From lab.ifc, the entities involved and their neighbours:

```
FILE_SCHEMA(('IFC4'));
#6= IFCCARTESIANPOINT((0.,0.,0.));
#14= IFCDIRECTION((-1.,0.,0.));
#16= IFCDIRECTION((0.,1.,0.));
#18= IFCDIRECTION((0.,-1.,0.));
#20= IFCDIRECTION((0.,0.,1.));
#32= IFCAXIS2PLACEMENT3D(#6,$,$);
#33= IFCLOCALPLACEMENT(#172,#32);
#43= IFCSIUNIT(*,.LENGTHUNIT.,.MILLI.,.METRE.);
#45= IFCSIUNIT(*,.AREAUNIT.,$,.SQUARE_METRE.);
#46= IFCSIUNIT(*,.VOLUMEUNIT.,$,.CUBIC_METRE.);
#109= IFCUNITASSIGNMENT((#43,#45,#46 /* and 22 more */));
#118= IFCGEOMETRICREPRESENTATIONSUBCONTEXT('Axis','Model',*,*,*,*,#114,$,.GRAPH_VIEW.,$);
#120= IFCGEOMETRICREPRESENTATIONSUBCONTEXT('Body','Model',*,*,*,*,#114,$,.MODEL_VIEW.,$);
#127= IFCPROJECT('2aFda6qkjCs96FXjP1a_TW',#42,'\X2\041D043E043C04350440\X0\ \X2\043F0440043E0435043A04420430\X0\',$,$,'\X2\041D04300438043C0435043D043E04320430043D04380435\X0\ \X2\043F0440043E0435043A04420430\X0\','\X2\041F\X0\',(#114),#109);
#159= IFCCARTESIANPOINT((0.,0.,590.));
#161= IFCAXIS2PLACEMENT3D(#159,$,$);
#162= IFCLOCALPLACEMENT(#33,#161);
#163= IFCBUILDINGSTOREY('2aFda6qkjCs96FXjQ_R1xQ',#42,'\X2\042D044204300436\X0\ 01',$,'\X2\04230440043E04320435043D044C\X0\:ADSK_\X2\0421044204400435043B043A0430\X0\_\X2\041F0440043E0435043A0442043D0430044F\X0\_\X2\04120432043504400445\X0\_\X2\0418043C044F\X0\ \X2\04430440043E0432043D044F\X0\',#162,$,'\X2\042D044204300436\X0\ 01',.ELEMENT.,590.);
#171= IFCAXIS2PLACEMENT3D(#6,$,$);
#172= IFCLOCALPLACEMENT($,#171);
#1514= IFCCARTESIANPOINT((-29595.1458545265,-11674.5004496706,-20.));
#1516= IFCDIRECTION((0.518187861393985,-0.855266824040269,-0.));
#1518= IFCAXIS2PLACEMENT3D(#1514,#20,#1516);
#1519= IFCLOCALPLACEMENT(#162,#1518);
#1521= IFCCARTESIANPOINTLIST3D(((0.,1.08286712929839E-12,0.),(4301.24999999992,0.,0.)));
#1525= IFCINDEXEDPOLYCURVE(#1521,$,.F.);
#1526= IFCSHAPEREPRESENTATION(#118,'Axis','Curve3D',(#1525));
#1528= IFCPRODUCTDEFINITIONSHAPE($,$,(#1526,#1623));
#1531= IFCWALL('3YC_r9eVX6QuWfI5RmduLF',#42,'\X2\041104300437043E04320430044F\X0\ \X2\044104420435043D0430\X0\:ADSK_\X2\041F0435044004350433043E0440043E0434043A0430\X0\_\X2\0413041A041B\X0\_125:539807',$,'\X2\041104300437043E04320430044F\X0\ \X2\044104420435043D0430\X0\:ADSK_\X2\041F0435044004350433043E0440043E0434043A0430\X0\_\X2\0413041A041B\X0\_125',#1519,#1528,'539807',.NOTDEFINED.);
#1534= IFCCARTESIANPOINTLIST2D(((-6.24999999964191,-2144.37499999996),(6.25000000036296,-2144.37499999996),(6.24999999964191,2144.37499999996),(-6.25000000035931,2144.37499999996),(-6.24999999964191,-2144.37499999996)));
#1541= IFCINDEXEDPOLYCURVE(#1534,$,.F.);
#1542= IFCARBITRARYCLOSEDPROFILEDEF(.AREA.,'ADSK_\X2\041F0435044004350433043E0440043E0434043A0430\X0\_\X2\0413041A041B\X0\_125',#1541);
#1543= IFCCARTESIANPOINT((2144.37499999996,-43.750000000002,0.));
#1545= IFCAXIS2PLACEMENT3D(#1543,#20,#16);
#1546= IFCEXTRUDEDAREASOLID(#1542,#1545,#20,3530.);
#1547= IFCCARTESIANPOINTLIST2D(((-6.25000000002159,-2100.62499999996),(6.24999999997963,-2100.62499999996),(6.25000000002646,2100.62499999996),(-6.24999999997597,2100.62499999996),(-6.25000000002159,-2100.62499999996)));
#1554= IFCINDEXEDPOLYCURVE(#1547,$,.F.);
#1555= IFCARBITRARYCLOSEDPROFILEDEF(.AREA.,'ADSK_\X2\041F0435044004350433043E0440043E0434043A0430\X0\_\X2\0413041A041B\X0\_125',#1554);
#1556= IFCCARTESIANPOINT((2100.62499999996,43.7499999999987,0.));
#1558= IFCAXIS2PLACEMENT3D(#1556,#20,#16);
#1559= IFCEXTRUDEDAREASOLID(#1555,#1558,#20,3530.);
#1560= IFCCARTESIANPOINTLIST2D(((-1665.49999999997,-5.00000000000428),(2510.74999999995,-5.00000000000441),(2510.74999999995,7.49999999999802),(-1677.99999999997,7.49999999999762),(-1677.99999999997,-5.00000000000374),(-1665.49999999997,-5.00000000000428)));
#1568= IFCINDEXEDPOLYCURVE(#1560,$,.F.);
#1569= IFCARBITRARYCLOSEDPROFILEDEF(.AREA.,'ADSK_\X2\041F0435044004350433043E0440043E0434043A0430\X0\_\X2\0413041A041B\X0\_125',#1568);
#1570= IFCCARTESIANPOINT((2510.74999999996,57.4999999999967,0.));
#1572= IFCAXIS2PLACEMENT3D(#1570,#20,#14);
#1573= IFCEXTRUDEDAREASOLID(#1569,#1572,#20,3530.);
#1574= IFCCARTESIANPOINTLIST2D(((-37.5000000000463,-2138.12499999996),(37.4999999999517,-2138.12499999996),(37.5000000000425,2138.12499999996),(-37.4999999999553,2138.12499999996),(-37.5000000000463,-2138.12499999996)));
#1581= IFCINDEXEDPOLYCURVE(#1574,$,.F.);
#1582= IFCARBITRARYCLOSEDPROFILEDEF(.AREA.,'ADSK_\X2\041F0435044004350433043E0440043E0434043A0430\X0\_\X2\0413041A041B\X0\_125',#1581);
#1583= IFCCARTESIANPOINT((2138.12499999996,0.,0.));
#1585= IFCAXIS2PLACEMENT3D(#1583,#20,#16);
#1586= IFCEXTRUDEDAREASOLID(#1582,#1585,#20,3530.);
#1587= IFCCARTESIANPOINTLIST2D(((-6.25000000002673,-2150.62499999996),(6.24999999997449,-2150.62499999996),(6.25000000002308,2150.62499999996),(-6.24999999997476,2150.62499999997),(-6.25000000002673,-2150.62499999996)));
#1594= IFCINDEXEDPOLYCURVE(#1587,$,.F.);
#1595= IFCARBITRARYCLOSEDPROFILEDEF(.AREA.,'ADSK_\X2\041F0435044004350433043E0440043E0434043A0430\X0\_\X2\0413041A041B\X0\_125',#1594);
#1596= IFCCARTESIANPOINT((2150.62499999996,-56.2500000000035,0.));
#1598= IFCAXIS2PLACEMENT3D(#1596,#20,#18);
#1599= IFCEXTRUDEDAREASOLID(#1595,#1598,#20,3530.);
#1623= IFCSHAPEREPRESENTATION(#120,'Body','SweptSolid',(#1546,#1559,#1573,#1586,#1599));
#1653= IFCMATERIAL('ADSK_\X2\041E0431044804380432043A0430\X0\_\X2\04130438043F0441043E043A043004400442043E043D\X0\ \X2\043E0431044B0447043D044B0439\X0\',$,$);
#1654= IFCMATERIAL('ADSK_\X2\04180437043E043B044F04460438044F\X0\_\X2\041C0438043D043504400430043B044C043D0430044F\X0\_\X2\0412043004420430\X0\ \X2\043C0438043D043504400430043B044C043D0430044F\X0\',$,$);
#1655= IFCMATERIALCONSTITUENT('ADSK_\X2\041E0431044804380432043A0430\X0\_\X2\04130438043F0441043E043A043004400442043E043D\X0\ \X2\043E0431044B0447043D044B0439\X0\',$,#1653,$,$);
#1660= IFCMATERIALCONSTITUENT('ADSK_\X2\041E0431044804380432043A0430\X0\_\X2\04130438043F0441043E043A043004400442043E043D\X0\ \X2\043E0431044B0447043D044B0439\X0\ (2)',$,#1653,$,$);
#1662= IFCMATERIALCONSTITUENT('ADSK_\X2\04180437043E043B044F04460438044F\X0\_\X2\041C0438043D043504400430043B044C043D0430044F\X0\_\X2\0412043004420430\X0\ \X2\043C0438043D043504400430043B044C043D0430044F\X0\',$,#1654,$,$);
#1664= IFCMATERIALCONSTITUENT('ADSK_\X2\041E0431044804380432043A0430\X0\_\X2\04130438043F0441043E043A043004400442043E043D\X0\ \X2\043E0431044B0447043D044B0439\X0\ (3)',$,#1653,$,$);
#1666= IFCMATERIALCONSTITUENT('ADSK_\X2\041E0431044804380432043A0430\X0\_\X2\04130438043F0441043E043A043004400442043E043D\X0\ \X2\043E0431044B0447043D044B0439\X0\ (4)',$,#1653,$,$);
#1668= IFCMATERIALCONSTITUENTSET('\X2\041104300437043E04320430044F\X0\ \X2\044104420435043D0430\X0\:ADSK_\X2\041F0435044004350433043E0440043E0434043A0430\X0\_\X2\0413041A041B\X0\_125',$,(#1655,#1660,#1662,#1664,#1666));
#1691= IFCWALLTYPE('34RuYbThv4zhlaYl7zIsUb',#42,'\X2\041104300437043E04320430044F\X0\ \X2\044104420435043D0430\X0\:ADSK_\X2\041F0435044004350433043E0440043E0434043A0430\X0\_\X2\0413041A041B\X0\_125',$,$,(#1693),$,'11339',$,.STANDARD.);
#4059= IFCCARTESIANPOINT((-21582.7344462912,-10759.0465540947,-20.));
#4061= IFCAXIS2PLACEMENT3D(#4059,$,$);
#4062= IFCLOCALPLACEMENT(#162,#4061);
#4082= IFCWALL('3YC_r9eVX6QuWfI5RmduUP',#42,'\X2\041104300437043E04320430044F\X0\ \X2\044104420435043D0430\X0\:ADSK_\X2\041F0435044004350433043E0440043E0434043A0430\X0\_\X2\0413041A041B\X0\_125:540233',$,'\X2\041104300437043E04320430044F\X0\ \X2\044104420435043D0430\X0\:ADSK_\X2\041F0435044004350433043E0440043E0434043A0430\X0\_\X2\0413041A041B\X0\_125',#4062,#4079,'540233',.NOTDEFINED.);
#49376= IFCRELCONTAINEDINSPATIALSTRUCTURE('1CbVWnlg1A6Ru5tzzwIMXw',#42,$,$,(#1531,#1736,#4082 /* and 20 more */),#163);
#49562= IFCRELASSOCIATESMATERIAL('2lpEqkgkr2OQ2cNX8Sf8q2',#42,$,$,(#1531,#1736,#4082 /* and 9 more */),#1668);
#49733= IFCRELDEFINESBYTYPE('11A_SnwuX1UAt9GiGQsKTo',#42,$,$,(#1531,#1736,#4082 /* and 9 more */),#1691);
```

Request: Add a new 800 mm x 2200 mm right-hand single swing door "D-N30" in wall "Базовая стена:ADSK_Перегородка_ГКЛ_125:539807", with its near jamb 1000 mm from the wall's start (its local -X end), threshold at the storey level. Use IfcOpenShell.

```python
import numpy as np
import ifcopenshell
import ifcopenshell.api.feature
import ifcopenshell.api.geometry
import ifcopenshell.api.root
import ifcopenshell.api.spatial
import ifcopenshell.geom
import ifcopenshell.util.element
import ifcopenshell.util.placement
import ifcopenshell.util.representation
import ifcopenshell.util.shape
import ifcopenshell.util.unit

model = ifcopenshell.open("lab.ifc")
unit_scale = ifcopenshell.util.unit.calculate_unit_scale(model)
settings = ifcopenshell.geom.settings()


def volume(element):
    """Net volume in cubic metres, openings subtracted."""
    shape = ifcopenshell.geom.create_shape(settings, element)
    return ifcopenshell.util.shape.get_volume(shape.geometry)


wall = model.by_id(1531)
storey = ifcopenshell.util.element.get_container(wall, ifc_class="IfcBuildingStorey")
context = ifcopenshell.util.representation.get_context(model, "Model", "Body", "MODEL_VIEW")
before = volume(wall)

width, height, from_end, sill = 0.8, 2.2, 1, 0.0  # metres

# The wall runs along its own X axis, and the end named is its -X end.
wall_shape = ifcopenshell.geom.create_shape(settings, wall)
x, y, z = ifcopenshell.util.shape.get_vertices(wall_shape.geometry).T
start = x.min() + from_end
face, thickness = float(y.min()), float(y.max() - y.min())
wall_matrix = ifcopenshell.util.placement.get_local_placement(wall.ObjectPlacement)
level = ifcopenshell.util.placement.get_local_placement(storey.ObjectPlacement)[2, 3]


def in_wall(x, y):
    """Placement at x, y metres in the wall's axes, at sill height."""
    matrix = wall_matrix.copy()
    matrix[:, 3] = wall_matrix @ np.array([x / unit_scale, y / unit_scale, 0.0, 1.0])
    matrix[2, 3] = level + sill / unit_scale
    return matrix


# Opening: a box that overshoots both wall faces by 50 mm.
opening = ifcopenshell.api.root.create_entity(model, ifc_class="IfcOpeningElement", predefined_type="OPENING")
box = ifcopenshell.api.geometry.add_wall_representation(
    model, context=context, length=width, height=height, thickness=thickness + 0.1
)
ifcopenshell.api.geometry.assign_representation(model, product=opening, representation=box)
ifcopenshell.api.geometry.edit_object_placement(model, product=opening, matrix=in_wall(start, face - 0.05), is_si=False)
ifcopenshell.api.feature.add_feature(model, feature=opening, element=wall)

door = ifcopenshell.api.root.create_entity(model, ifc_class="IfcDoor", name="D-N30", predefined_type="DOOR")
door.OverallWidth, door.OverallHeight = width / unit_scale, height / unit_scale
door.OperationType = "SINGLE_SWING_RIGHT"
body = ifcopenshell.api.geometry.add_door_representation(
    model,
    context=context,
    overall_width=door.OverallWidth,
    overall_height=door.OverallHeight,
    operation_type="SINGLE_SWING_RIGHT",
    lining_properties={"LiningDepth": thickness / unit_scale, "ThresholdDepth": thickness / unit_scale},
)
ifcopenshell.api.geometry.assign_representation(model, product=door, representation=body)
ifcopenshell.api.spatial.assign_container(model, products=[door], relating_structure=storey)
ifcopenshell.api.feature.add_filling(model, opening=opening, element=door)

# The lining spans the wall, so the door starts at the wall face.
ifcopenshell.api.geometry.edit_object_placement(model, product=door, matrix=in_wall(start, face), is_si=False)

after = volume(wall)

print(f"wall volume {before:.3f} -> {after:.3f} m3")

model.write("lab_v2.ifc")
```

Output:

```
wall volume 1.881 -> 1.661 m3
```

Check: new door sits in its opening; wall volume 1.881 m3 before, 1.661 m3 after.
